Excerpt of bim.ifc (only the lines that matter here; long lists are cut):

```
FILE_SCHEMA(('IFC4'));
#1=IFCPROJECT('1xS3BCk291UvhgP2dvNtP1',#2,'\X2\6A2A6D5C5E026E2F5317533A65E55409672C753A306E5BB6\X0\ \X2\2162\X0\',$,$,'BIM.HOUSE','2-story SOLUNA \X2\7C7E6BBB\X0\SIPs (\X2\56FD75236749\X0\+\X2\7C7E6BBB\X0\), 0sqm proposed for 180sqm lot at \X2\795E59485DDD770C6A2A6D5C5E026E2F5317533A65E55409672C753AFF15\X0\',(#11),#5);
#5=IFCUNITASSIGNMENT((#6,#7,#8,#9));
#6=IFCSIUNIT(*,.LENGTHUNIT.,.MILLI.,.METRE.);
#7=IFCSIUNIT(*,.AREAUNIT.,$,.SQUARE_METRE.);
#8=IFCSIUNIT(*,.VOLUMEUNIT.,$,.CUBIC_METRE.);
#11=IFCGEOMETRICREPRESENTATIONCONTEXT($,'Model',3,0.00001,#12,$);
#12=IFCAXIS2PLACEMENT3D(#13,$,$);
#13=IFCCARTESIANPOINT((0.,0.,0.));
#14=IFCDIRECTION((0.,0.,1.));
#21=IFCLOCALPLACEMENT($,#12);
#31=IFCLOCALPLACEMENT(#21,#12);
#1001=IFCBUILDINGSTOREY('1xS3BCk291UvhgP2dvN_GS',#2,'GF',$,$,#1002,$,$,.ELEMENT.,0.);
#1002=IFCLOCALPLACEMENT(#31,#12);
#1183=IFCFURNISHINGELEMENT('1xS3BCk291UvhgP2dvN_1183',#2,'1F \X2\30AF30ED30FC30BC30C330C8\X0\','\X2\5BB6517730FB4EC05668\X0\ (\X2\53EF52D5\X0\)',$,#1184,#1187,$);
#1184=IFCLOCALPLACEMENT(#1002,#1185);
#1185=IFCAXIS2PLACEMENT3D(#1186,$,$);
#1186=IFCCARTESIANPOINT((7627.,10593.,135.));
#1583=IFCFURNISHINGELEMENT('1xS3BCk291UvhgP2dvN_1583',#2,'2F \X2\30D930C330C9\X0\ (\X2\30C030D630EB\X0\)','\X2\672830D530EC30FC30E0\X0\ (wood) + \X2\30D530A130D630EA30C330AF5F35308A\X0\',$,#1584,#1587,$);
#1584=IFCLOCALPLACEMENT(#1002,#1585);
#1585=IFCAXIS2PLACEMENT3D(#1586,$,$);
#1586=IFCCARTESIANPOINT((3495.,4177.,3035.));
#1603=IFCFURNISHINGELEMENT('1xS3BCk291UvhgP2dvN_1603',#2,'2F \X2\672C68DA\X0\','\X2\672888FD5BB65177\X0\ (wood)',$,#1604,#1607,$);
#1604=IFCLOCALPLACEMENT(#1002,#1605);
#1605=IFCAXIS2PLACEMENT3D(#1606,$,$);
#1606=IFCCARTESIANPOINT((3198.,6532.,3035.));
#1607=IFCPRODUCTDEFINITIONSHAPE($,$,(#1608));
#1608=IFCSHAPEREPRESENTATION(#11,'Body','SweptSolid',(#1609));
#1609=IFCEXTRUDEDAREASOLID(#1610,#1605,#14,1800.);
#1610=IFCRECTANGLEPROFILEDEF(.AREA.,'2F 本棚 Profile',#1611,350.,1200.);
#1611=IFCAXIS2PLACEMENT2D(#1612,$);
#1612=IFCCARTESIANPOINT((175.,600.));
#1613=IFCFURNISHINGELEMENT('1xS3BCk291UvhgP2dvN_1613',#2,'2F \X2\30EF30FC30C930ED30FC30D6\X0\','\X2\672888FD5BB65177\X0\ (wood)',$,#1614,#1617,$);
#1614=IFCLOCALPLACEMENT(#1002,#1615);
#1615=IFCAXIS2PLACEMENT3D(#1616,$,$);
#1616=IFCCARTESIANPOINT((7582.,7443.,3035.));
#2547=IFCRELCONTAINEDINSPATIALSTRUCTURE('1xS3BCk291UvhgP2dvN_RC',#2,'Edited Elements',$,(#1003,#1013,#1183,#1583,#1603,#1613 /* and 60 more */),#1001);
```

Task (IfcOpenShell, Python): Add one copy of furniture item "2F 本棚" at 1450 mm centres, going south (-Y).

```python
import numpy as np
import ifcopenshell
import ifcopenshell.api.geometry
import ifcopenshell.api.root
import ifcopenshell.util.element
import ifcopenshell.util.placement
import ifcopenshell.util.unit

model = ifcopenshell.open("bim.ifc")
unit_scale = ifcopenshell.util.unit.calculate_unit_scale(model)


def reuse_history(source, copy):
    """copy_class also copies each property set's owner history, people and application; keep the originals."""
    for rel in copy.IsDefinedBy:
        if rel.is_a("IfcRelDefinesByProperties") and (history := rel.RelatingPropertyDefinition.OwnerHistory):
            rel.RelatingPropertyDefinition.OwnerHistory = source.OwnerHistory
            ifcopenshell.util.element.remove_deep2(model, history)


source = model.by_guid("1xS3BCk291UvhgP2dvN_1603")
base = ifcopenshell.util.placement.get_local_placement(source.ObjectPlacement)
step = np.array([0.0, -1.0, 0.0]) * 1.45 / unit_scale

for i in range(1, 2):
    copy = ifcopenshell.api.root.copy_class(model, product=source)
    copy.Representation = ifcopenshell.util.element.copy_deep(
        model, source.Representation, exclude=["IfcGeometricRepresentationContext", "IfcRepresentationMap"]
    )
    reuse_history(source, copy)
    matrix = base.copy()
    matrix[:3, 3] += i * step
    print("added at", matrix[:3, 3].round(3) + 0.0)
    ifcopenshell.api.geometry.edit_object_placement(model, product=copy, matrix=matrix, is_si=False)

model.write("bim_rev.ifc")
```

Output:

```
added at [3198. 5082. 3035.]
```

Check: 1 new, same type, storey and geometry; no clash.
